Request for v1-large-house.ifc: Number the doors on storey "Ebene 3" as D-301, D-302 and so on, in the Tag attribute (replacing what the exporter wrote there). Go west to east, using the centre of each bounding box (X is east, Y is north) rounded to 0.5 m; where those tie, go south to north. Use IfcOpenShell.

First a look at what the model holds.

```python
import ifcopenshell
import ifcopenshell.util.element
import ifcopenshell.util.placement

model = ifcopenshell.open("v1-large-house.ifc")
print(model.schema)
storey = next(s for s in model.by_type("IfcBuildingStorey") if s.Name == "Ebene 3")
doors = [e for e in ifcopenshell.util.element.get_decomposition(storey) if e.is_a("IfcDoor")]
for e in sorted(doors, key=lambda e: e.id()):
    origin = ifcopenshell.util.placement.get_local_placement(e.ObjectPlacement)[:3, 3]
    print(e.id(), e.Tag, e.Name, origin.round(2) + 0.0, sep=" | ")
```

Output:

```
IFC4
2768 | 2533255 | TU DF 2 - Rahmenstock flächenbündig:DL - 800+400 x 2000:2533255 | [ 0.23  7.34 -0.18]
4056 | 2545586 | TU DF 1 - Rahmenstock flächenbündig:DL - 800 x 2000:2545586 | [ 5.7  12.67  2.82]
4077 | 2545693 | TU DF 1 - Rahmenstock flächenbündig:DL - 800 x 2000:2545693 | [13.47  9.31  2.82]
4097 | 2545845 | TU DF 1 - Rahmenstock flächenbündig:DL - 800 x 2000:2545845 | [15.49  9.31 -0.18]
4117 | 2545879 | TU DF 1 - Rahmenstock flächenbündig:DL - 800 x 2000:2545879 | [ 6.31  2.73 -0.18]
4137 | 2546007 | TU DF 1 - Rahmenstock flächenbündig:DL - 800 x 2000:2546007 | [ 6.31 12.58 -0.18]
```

```python
import ifcopenshell
import ifcopenshell.geom
import ifcopenshell.util.element
import ifcopenshell.util.shape

model = ifcopenshell.open("v1-large-house.ifc")
settings = ifcopenshell.geom.settings()
settings.set("use-world-coords", True)


def centre(element):
    shape = ifcopenshell.geom.create_shape(settings, element)
    return ifcopenshell.util.shape.get_bbox_centroid(shape.geometry)


storey = next(s for s in model.by_type("IfcBuildingStorey") if s.Name == "Ebene 3")
doors = [e for e in ifcopenshell.util.element.get_decomposition(storey) if e.is_a("IfcDoor")]

# Insertion points can sit at a corner or the storey origin, so sort by the geometry (in metres).
centres = {e: centre(e) for e in doors}
doors.sort(key=lambda e: (round(centres[e][0] / 0.5), centres[e][1]))

for i, e in enumerate(doors, start=1):
    number = f"D-3{i:02d}"
    e.Tag = number
    print(e.id(), number)

model.write("v1-large-house_v2.ifc")
```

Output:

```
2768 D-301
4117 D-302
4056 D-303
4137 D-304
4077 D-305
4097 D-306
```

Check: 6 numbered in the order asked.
